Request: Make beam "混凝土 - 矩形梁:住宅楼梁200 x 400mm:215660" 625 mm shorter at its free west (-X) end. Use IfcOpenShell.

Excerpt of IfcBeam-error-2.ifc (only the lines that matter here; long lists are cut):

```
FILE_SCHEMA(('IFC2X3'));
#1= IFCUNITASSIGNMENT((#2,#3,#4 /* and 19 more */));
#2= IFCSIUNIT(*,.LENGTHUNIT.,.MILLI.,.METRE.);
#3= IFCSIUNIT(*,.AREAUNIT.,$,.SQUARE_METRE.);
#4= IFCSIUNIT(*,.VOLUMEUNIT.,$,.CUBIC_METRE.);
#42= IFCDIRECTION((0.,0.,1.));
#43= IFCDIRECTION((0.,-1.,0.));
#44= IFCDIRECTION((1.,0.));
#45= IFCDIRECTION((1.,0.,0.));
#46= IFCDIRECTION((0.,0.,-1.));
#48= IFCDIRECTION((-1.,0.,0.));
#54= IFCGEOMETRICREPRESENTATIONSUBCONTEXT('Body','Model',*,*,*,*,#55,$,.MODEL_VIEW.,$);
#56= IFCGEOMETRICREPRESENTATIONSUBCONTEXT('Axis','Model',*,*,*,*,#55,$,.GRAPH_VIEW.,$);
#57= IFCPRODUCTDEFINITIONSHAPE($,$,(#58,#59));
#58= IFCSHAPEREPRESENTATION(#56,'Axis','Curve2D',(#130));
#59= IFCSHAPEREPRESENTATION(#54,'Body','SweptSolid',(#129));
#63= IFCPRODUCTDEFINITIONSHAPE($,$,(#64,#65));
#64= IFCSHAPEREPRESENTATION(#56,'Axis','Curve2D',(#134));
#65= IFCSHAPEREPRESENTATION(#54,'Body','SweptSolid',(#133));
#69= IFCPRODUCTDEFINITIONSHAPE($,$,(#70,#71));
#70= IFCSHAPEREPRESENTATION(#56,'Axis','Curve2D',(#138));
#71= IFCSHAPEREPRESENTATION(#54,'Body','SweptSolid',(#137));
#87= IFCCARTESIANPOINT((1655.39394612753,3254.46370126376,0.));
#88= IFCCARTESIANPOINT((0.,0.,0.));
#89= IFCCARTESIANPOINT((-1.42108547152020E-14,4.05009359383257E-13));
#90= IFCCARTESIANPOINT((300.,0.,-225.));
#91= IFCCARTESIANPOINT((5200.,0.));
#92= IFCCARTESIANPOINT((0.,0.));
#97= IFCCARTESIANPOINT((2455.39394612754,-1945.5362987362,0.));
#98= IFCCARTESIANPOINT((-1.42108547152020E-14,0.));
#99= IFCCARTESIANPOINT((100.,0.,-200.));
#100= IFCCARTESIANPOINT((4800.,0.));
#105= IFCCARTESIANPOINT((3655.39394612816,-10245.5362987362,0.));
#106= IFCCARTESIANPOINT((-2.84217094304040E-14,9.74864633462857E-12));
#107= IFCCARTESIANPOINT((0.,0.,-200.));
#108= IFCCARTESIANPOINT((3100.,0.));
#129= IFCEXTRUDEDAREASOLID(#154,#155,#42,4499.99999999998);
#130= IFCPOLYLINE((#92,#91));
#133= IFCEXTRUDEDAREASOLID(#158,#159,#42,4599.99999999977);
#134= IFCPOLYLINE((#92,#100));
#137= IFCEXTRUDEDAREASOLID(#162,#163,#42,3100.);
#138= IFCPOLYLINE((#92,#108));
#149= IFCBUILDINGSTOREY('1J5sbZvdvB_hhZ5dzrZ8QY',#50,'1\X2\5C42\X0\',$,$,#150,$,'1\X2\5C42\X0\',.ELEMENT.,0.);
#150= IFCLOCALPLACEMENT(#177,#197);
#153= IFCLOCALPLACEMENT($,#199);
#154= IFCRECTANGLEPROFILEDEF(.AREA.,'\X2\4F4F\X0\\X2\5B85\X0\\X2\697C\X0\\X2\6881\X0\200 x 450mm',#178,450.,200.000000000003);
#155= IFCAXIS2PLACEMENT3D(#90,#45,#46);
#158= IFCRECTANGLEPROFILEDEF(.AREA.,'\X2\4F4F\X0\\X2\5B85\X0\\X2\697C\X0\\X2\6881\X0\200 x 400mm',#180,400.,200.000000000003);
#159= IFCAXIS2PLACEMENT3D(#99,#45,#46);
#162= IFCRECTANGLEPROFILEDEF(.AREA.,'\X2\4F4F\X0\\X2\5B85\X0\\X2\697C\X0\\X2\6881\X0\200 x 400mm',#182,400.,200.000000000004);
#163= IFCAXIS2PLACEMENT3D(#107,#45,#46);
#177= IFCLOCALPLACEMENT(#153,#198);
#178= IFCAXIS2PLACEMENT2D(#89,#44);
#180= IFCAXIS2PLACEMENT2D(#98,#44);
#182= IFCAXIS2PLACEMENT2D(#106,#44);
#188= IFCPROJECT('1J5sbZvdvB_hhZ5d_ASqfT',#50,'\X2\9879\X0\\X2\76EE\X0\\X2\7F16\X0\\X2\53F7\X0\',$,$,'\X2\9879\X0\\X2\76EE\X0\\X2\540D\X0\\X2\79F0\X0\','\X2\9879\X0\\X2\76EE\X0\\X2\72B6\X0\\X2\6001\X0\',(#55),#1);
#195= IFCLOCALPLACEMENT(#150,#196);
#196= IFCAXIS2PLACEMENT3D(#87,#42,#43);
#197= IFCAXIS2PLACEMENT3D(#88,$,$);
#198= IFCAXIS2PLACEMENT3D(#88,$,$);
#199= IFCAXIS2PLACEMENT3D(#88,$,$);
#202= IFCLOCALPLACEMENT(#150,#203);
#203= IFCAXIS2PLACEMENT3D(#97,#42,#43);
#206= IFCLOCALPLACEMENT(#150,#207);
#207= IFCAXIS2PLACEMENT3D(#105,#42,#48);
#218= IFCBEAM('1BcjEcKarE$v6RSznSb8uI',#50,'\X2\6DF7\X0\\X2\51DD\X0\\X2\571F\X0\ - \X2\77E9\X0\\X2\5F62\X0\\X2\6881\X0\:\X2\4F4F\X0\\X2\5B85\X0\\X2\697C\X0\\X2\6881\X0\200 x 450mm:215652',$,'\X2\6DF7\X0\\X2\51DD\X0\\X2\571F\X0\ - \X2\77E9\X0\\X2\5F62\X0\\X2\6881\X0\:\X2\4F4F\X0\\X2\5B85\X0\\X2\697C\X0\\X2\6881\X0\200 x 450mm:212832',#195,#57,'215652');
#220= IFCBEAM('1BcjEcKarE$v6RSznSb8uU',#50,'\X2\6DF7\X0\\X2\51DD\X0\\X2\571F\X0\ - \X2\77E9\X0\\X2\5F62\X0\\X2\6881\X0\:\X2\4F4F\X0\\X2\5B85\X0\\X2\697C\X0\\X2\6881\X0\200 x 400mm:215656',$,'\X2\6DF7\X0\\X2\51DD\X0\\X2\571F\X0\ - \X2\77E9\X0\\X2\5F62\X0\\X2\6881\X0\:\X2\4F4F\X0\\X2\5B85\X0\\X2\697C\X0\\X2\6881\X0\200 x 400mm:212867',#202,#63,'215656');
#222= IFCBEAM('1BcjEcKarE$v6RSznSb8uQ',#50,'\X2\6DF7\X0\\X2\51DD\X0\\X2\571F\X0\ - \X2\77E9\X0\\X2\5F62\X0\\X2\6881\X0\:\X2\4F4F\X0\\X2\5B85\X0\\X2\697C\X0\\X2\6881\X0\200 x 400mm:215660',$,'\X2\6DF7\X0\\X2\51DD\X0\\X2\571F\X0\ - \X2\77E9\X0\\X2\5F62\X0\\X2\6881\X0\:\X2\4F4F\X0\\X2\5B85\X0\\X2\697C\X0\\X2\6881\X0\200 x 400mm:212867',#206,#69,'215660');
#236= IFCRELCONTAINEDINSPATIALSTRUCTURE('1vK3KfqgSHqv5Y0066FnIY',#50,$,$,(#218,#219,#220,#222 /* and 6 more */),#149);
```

```python
import numpy as np
import ifcopenshell
import ifcopenshell.util.representation
import ifcopenshell.util.unit

model = ifcopenshell.open("IfcBeam-error-2.ifc")
unit_scale = ifcopenshell.util.unit.calculate_unit_scale(model)

member = model.by_id(222)
change = -0.625 / unit_scale

# The extrusion runs towards the end named, so only its depth changes.
body = ifcopenshell.util.representation.get_representation(member, "Model", "Body")
solid = body.Items[0]
old_length = solid.Depth
solid.Depth += change

# Move the axis end point with it.
axis = next(r for r in member.Representation.Representations if r.RepresentationIdentifier == "Axis").Items[0]
start, end = (np.array(p.Coordinates) for p in axis.Points)
end = end + (end - start) / np.linalg.norm(end - start) * change
point = model.createIfcCartesianPoint(end.tolist())
axis.Points = [axis.Points[0], point]

print(f"length {old_length:g} -> {solid.Depth:g}")

model.write("IfcBeam-error-2_updated.ifc")
```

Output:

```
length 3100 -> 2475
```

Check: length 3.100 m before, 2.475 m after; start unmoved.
